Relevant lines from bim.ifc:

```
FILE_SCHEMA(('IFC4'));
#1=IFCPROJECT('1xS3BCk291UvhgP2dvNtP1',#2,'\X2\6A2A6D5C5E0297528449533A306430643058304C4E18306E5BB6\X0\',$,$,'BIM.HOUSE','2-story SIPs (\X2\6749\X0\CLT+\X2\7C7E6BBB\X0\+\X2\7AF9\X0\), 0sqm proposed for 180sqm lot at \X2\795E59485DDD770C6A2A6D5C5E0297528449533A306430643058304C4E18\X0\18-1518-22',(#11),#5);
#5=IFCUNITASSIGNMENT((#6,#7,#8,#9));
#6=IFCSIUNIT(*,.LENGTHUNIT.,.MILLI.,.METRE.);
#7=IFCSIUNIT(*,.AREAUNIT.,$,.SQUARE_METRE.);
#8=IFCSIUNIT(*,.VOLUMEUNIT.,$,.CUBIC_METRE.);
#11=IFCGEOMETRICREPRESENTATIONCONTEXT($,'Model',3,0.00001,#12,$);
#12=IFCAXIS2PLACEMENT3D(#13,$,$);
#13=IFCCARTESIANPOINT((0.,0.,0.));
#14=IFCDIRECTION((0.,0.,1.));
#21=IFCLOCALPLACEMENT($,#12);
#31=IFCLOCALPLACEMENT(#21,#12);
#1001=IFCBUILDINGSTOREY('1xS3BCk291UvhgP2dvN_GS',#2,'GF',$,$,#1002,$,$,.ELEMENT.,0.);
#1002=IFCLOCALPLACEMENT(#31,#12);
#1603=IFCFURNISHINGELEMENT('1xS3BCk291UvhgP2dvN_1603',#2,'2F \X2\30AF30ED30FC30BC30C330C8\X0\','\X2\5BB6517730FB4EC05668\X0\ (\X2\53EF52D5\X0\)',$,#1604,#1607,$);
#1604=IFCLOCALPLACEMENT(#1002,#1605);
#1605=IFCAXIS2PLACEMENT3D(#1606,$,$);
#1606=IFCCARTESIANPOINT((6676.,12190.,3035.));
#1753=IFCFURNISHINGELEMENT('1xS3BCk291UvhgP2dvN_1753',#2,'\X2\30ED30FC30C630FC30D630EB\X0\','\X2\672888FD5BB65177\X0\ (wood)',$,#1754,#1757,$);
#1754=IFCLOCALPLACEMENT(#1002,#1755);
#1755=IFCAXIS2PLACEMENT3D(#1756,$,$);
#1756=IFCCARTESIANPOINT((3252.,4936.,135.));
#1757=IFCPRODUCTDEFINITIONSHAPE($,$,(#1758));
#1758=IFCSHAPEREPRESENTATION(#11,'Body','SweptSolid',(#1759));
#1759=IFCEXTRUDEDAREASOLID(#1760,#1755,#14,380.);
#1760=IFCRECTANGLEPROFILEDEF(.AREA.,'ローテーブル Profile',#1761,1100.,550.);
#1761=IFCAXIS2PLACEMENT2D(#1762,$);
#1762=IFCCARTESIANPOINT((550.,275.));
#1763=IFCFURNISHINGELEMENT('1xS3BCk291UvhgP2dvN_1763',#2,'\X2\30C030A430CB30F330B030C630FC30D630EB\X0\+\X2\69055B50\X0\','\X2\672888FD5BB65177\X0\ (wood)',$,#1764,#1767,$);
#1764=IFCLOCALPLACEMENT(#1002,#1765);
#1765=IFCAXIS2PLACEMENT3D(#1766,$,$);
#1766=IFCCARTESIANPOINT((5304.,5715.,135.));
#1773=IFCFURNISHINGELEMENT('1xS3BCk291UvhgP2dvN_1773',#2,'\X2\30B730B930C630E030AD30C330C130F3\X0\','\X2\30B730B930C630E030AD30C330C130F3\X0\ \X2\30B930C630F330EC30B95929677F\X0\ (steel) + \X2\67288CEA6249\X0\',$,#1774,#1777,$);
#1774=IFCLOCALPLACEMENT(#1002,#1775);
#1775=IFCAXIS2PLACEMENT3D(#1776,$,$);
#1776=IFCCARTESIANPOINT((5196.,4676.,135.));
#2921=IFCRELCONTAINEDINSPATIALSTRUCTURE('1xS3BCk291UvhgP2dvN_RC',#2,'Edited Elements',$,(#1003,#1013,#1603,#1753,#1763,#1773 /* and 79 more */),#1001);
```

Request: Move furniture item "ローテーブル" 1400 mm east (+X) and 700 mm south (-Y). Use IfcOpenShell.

```python
import ifcopenshell
import ifcopenshell.api.geometry
import ifcopenshell.util.placement
import ifcopenshell.util.unit

model = ifcopenshell.open("bim.ifc")
unit_scale = ifcopenshell.util.unit.calculate_unit_scale(model)

item = model.by_id(1753)
matrix = ifcopenshell.util.placement.get_local_placement(item.ObjectPlacement)
matrix[0, 3] += 1.4 / unit_scale
matrix[1, 3] -= 0.7 / unit_scale
ifcopenshell.api.geometry.edit_object_placement(model, product=item, matrix=matrix, is_si=False)

print(ifcopenshell.util.placement.get_local_placement(item.ObjectPlacement).round(3) + 0.0)

model.write("bim_updated.ifc")
```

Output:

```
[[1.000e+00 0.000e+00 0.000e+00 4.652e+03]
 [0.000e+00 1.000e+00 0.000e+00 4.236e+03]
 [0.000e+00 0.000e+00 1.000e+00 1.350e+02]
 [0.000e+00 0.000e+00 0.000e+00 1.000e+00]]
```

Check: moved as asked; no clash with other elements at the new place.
